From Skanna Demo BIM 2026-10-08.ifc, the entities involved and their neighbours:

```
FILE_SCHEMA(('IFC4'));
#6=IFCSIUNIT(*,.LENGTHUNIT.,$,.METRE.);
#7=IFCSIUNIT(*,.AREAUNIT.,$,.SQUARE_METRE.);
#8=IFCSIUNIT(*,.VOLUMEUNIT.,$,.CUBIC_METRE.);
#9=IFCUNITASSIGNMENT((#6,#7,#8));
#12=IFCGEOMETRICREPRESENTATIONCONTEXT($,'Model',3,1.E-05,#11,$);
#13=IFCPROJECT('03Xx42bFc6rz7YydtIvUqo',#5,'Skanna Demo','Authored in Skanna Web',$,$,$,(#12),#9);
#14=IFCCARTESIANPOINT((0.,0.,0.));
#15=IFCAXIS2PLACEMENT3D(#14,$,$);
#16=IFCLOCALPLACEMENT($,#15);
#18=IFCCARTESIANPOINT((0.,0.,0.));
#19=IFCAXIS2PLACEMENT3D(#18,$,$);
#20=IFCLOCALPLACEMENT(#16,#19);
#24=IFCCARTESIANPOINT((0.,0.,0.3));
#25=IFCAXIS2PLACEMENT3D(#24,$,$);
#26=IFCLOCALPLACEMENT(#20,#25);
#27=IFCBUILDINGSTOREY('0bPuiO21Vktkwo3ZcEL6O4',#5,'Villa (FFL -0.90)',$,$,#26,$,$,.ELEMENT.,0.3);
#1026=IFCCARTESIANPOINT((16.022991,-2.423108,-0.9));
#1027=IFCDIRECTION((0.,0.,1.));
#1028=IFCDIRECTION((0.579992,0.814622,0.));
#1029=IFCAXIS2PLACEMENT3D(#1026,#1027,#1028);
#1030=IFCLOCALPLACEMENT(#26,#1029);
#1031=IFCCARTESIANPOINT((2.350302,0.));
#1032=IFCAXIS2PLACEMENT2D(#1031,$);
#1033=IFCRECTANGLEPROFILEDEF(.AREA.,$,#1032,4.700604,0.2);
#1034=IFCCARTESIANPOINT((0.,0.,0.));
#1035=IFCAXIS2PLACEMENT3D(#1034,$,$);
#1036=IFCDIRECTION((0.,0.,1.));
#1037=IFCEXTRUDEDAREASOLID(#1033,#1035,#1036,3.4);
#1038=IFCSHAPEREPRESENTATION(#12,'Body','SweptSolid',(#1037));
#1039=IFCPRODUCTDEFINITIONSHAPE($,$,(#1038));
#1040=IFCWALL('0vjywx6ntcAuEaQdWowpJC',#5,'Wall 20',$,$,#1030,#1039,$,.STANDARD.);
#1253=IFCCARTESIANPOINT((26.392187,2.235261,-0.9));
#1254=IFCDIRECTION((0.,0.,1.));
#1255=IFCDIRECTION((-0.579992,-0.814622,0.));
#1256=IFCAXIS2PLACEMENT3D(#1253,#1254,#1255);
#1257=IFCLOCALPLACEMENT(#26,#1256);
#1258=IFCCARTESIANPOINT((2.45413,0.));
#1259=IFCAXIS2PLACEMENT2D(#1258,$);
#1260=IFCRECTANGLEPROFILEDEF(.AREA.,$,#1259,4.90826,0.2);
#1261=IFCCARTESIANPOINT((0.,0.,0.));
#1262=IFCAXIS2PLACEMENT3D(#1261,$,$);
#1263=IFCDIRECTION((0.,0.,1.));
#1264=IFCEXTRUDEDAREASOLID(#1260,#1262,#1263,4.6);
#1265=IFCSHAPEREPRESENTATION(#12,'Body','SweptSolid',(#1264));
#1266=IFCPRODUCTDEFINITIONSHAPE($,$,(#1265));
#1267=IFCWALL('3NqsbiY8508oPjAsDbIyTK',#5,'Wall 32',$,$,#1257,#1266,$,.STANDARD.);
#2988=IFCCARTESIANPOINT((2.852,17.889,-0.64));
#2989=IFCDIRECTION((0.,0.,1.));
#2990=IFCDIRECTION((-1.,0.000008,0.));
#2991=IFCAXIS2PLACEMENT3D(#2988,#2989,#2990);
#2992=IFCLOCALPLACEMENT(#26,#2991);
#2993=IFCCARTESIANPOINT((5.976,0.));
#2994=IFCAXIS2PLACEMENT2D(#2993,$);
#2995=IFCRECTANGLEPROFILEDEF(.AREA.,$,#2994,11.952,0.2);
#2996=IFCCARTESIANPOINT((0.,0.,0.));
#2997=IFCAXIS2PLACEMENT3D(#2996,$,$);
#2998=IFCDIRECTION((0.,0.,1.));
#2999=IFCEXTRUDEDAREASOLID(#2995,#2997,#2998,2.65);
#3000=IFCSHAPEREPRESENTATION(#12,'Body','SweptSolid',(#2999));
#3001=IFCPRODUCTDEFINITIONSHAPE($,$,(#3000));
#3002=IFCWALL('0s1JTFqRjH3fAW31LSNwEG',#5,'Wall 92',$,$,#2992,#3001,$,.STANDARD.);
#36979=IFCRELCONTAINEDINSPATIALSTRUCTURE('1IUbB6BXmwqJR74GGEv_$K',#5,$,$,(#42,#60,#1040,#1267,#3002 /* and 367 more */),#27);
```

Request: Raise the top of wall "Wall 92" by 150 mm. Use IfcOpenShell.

```python
import ifcopenshell
import ifcopenshell.geom
import ifcopenshell.util.shape
import ifcopenshell.util.unit

model = ifcopenshell.open("Skanna Demo BIM 2026-10-08.ifc")
unit_scale = ifcopenshell.util.unit.calculate_unit_scale(model)
settings = ifcopenshell.geom.settings()


def volume(element):
    """Net volume in cubic metres, openings subtracted."""
    shape = ifcopenshell.geom.create_shape(settings, element)
    return ifcopenshell.util.shape.get_volume(shape.geometry)


wall = model.by_guid("0s1JTFqRjH3fAW31LSNwEG")
before = volume(wall)

body = next(r for r in wall.Representation.Representations if r.RepresentationIdentifier == "Body")
solid = body.Items[0]
old_height = solid.Depth
solid.Depth += 0.15 / unit_scale
after = volume(wall)

print(f"height {old_height:g} -> {solid.Depth:g}, volume {before:.3f} -> {after:.3f} m3")

model.write("Skanna Demo BIM 2026-10-08_updated.ifc")
```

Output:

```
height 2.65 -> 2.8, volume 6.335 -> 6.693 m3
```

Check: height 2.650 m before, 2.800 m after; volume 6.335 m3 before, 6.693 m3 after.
